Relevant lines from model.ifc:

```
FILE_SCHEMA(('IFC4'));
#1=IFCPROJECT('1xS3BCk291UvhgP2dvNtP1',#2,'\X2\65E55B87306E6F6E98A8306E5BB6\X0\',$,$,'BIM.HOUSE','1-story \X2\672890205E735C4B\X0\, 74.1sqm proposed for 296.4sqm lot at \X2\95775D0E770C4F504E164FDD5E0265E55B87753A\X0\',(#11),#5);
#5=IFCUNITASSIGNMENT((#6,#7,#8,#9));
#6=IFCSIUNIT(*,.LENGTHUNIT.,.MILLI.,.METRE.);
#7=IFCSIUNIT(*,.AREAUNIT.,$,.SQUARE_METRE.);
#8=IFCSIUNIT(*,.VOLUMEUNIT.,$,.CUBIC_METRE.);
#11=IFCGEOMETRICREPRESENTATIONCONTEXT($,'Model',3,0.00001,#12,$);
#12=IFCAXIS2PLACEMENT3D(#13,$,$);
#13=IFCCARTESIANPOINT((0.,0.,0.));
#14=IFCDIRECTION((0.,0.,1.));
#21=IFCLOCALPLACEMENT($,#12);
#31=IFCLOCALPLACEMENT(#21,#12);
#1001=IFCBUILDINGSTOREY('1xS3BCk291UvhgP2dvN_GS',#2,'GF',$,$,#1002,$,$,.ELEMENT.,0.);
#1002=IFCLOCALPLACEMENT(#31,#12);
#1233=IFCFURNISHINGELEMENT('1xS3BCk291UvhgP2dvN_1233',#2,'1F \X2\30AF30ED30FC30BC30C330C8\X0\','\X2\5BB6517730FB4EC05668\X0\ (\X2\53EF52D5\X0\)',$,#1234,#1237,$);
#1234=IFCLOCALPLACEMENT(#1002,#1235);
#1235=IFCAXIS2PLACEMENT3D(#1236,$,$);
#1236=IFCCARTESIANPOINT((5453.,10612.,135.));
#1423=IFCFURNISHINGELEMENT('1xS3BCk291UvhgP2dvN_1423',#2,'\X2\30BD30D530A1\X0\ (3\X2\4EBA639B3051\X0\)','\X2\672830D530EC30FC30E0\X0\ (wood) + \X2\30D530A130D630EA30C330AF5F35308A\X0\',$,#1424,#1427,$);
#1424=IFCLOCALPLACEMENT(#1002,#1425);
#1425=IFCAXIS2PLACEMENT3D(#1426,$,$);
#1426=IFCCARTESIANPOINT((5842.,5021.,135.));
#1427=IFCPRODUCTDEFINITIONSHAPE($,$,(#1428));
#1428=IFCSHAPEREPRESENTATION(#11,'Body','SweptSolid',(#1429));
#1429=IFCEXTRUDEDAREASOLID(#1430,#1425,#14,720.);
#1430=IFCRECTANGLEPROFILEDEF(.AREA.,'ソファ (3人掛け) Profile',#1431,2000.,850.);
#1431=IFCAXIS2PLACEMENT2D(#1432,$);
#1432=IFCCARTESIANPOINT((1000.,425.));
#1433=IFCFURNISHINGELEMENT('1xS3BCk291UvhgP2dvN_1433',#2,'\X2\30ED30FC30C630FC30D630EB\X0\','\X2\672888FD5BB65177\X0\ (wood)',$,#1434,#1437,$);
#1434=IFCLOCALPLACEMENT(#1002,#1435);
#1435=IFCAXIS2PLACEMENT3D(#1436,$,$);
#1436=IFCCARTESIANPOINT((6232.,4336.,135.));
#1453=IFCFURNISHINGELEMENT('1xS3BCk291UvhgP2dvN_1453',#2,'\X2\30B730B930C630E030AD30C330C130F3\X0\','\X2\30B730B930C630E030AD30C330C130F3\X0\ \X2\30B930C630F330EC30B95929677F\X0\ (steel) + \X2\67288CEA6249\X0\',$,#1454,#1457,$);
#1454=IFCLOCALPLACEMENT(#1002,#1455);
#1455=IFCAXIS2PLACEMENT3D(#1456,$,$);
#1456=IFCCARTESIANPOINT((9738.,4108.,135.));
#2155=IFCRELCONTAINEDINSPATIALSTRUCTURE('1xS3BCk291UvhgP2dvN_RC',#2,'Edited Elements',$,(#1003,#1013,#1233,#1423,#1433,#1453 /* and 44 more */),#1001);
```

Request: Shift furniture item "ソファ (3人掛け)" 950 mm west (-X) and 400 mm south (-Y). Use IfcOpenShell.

```python
import ifcopenshell
import ifcopenshell.api.geometry
import ifcopenshell.util.placement

model = ifcopenshell.open("model.ifc")

item = model.by_guid("1xS3BCk291UvhgP2dvN_1423")
matrix = ifcopenshell.util.placement.get_local_placement(item.ObjectPlacement)
matrix[0, 3] -= 950.0
matrix[1, 3] -= 400.0
ifcopenshell.api.geometry.edit_object_placement(model, product=item, matrix=matrix, is_si=False)

print(ifcopenshell.util.placement.get_local_placement(item.ObjectPlacement).round(3) + 0.0)

model.write("model_rev.ifc")
```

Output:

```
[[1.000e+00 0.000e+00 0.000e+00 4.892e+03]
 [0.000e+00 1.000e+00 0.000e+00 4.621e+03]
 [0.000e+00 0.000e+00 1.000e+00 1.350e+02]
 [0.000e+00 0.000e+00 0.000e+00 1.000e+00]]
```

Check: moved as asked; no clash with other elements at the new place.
